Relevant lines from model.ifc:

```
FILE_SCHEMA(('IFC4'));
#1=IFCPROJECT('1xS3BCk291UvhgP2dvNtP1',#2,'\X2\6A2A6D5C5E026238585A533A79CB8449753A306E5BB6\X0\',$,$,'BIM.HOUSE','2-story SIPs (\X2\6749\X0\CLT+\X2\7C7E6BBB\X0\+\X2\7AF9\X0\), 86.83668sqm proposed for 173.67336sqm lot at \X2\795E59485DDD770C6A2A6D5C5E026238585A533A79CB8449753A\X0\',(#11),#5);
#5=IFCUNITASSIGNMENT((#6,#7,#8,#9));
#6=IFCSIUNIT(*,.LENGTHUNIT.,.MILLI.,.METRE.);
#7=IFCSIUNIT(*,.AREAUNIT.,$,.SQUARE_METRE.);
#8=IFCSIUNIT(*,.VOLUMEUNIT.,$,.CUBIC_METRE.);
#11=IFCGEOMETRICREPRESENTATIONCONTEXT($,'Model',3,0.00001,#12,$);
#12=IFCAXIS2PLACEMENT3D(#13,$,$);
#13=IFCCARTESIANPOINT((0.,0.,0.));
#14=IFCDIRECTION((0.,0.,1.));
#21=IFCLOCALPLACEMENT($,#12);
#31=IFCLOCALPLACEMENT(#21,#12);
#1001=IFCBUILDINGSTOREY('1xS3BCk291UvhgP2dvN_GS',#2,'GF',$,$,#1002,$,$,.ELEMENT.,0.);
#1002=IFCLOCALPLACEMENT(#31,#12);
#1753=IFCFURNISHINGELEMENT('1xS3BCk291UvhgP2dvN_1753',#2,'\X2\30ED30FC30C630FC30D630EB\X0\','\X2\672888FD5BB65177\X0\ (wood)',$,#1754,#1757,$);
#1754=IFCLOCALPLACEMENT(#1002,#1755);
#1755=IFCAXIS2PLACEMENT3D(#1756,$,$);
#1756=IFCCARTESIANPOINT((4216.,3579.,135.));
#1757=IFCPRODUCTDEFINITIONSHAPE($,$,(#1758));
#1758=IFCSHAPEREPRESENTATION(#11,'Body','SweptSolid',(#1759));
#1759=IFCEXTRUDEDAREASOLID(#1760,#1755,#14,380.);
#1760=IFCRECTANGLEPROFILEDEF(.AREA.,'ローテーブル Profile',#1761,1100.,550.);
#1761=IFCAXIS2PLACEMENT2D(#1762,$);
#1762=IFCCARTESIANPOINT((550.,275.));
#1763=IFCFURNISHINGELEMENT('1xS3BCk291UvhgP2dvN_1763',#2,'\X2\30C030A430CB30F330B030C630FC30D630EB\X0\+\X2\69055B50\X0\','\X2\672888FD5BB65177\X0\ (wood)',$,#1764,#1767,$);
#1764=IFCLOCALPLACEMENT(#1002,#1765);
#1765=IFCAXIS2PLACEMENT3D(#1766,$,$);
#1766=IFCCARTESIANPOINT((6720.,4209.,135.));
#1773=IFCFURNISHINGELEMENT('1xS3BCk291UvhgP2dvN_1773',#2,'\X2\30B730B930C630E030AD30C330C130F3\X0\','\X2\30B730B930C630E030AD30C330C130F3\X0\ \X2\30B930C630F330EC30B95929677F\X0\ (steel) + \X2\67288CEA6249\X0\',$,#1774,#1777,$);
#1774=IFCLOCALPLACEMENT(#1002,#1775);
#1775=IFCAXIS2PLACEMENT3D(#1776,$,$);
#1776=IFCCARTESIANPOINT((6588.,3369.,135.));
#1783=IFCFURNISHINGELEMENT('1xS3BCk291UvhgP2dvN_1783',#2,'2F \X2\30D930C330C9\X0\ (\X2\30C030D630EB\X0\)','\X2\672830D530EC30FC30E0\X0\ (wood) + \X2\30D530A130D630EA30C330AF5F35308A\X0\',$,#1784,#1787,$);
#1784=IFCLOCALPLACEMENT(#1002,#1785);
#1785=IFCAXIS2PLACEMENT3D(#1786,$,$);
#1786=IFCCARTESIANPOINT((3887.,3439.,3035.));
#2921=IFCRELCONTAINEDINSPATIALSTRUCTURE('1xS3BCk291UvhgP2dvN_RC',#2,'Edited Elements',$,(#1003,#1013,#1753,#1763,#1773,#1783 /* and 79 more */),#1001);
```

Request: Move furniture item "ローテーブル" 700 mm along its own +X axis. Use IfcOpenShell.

```python
import ifcopenshell
import ifcopenshell.api.geometry
import ifcopenshell.util.placement
import ifcopenshell.util.unit

model = ifcopenshell.open("model.ifc")
unit_scale = ifcopenshell.util.unit.calculate_unit_scale(model)

item = model.by_guid("1xS3BCk291UvhgP2dvN_1753")
matrix = ifcopenshell.util.placement.get_local_placement(item.ObjectPlacement)
matrix[:3, 3] += matrix[:3, 0] * 0.7 / unit_scale
ifcopenshell.api.geometry.edit_object_placement(model, product=item, matrix=matrix, is_si=False)

print(ifcopenshell.util.placement.get_local_placement(item.ObjectPlacement).round(3) + 0.0)

model.write("model_updated.ifc")
```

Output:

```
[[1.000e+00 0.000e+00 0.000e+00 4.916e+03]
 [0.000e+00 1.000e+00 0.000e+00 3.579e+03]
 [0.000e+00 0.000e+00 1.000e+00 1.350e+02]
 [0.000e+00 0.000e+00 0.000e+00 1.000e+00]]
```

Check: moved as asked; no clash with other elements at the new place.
